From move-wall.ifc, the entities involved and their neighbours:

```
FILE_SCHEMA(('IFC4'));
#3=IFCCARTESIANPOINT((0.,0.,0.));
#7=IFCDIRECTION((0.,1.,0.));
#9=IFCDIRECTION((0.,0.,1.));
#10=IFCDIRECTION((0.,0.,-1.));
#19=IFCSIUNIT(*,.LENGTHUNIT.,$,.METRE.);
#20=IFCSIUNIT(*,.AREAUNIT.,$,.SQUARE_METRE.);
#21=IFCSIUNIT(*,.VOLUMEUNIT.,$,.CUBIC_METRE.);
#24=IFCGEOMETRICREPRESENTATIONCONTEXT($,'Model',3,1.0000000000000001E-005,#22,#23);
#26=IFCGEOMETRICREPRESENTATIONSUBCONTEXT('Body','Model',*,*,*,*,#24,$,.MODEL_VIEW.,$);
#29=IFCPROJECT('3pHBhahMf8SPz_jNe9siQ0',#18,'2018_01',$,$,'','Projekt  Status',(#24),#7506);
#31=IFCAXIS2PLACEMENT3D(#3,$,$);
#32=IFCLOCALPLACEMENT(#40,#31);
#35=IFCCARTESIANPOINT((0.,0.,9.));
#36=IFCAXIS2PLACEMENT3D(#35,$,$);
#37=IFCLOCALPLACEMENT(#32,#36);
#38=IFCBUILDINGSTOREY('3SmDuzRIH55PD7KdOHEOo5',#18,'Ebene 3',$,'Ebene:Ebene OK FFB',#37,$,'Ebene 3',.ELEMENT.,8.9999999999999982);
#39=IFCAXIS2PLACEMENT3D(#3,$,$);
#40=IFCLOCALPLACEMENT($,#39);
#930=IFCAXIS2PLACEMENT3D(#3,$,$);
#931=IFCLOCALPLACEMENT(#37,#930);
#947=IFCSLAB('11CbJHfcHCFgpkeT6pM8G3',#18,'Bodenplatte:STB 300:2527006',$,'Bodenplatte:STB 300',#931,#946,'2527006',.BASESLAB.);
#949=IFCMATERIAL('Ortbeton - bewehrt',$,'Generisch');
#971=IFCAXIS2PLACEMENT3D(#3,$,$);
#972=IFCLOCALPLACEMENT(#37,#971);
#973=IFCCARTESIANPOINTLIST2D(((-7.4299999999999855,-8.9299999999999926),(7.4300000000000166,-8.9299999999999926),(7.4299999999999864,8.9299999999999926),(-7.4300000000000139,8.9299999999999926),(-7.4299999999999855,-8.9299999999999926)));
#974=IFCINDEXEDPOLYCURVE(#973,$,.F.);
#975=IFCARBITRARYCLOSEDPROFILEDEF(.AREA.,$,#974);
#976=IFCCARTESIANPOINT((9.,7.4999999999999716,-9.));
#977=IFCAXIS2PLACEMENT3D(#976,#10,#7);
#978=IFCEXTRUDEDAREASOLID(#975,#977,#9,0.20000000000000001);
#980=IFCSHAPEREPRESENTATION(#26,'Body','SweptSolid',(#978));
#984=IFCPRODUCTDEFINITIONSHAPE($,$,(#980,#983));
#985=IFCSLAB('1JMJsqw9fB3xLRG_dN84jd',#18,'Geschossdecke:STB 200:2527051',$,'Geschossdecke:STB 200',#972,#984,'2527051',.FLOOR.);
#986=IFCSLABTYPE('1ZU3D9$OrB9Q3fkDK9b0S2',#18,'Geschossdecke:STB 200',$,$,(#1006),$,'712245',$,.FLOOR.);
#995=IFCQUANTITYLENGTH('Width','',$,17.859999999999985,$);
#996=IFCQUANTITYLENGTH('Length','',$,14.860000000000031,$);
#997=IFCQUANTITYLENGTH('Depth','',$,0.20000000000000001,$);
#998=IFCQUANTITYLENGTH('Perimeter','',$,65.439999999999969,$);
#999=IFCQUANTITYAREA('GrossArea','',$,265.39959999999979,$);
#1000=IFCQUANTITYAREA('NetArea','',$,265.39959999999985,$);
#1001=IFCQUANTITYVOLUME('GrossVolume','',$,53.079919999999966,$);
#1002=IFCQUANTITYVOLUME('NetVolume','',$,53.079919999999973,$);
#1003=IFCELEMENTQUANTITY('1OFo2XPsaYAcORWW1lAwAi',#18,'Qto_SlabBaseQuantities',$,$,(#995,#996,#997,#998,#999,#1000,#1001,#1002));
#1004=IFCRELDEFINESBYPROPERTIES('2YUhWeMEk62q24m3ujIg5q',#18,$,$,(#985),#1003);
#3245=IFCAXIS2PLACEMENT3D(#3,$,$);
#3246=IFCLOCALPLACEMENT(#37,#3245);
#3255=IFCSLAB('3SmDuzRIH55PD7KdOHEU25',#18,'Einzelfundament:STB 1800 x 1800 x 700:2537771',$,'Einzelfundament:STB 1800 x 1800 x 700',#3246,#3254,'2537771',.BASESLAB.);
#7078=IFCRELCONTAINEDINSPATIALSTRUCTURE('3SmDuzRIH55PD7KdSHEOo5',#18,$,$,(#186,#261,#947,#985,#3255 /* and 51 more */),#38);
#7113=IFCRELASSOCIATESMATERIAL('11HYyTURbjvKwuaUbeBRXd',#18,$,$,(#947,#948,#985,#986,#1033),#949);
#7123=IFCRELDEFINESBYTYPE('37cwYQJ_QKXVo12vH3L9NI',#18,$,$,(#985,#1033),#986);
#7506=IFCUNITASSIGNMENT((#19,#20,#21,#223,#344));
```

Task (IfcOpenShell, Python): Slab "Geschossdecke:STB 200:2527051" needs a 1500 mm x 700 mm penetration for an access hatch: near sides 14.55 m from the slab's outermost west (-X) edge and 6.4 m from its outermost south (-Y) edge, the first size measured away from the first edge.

```python
import numpy as np
import ifcopenshell
import ifcopenshell.api.feature
import ifcopenshell.api.geometry
import ifcopenshell.api.pset
import ifcopenshell.api.root
import ifcopenshell.geom
import ifcopenshell.util.element
import ifcopenshell.util.placement
import ifcopenshell.util.representation
import ifcopenshell.util.shape
import ifcopenshell.util.unit

model = ifcopenshell.open("move-wall.ifc")
unit_scale = ifcopenshell.util.unit.calculate_unit_scale(model)
area_scale = ifcopenshell.util.unit.calculate_unit_scale(model, "AREAUNIT")
volume_scale = ifcopenshell.util.unit.calculate_unit_scale(model, "VOLUMEUNIT")
settings = ifcopenshell.geom.settings()


def volume(element):
    """Net volume in cubic metres, openings subtracted."""
    shape = ifcopenshell.geom.create_shape(settings, element)
    return ifcopenshell.util.shape.get_volume(shape.geometry)


slab = model.by_guid("1JMJsqw9fB3xLRG_dN84jd")
before = volume(slab)

# Extent in the slab's own axes, in metres. The edges named are its -X and -Y sides.
slab_shape = ifcopenshell.geom.create_shape(settings, slab)
vertices = ifcopenshell.util.shape.get_vertices(slab_shape.geometry)
x_min, y_min, bottom = vertices.min(axis=0)
top = vertices[:, 2].max()

opening = ifcopenshell.api.root.create_entity(model, ifc_class="IfcOpeningElement", name="Access hatch opening", predefined_type="OPENING")
context = ifcopenshell.util.representation.get_context(model, "Model", "Body", "MODEL_VIEW")
width, depth = 1.5, 0.7
outline = [(0.0, 0.0), (width, 0.0), (width, depth), (0.0, depth), (0.0, 0.0)]
# Overshoot both faces by 50 mm so the cut is clean.
shape = ifcopenshell.api.geometry.add_slab_representation(
    model, context=context, depth=top - bottom + 0.1, polyline=outline
)
ifcopenshell.api.geometry.assign_representation(model, product=opening, representation=shape)

matrix = ifcopenshell.util.placement.get_local_placement(slab.ObjectPlacement)
matrix[:, 3] = matrix @ np.append(np.array([x_min + 14.55, y_min + 6.4, bottom - 0.05]) / unit_scale, 1.0)
ifcopenshell.api.geometry.edit_object_placement(model, product=opening, matrix=matrix, is_si=False)
ifcopenshell.api.feature.add_feature(model, feature=opening, element=slab)

after = volume(slab)

# Update the slab's stored quantities.
qto = model.by_id(ifcopenshell.util.element.get_pset(slab, "Qto_SlabBaseQuantities", should_inherit=False)["id"])
ifcopenshell.api.pset.edit_qto(model, qto=qto, properties={
    "NetArea": after / (top - bottom) / area_scale,
    "NetVolume": after / volume_scale,
})

print(f"slab volume {before:.3f} -> {after:.3f} m3")

model.write("move-wall-out.ifc")
```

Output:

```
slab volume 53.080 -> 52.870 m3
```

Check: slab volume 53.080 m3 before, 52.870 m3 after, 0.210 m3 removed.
